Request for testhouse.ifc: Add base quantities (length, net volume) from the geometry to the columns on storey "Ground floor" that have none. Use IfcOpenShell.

First a look at what the model holds.

```python
import ifcopenshell
import ifcopenshell.util.element
import ifcopenshell.util.unit

model = ifcopenshell.open("testhouse.ifc")
print(model.schema)
for unit_type in ("LENGTHUNIT", "AREAUNIT", "VOLUMEUNIT"):
    print(unit_type, ifcopenshell.util.unit.calculate_unit_scale(model, unit_type))
storey = next(s for s in model.by_type("IfcBuildingStorey") if s.Name == "Ground floor")
columns = [e for e in ifcopenshell.util.element.get_decomposition(storey) if e.is_a("IfcColumn")]
for e in sorted(columns, key=lambda e: e.id()):
    print(e.id(), e.is_a(), e.Name, list(ifcopenshell.util.element.get_psets(e, qtos_only=True)), sep=" | ")
```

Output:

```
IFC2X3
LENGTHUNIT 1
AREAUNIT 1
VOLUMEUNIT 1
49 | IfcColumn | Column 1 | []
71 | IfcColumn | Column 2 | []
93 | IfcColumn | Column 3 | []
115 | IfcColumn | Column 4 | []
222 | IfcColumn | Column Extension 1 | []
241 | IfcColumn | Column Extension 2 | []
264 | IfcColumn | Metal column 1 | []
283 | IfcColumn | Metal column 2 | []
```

```python
import ifcopenshell
import ifcopenshell.api.pset
import ifcopenshell.geom
import ifcopenshell.util.element
import ifcopenshell.util.shape
import ifcopenshell.util.unit

model = ifcopenshell.open("testhouse.ifc")
unit_scale = ifcopenshell.util.unit.calculate_unit_scale(model)
volume_scale = ifcopenshell.util.unit.calculate_unit_scale(model, "VOLUMEUNIT")
settings = ifcopenshell.geom.settings()

storey = next(s for s in model.by_type("IfcBuildingStorey") if s.Name == "Ground floor")
columns = [e for e in ifcopenshell.util.element.get_decomposition(storey) if e.is_a("IfcColumn")]

for e in sorted(columns, key=lambda e: e.id()):
    if ifcopenshell.util.element.get_psets(e, qtos_only=True, should_inherit=False):
        continue
    # Geometry comes back in metres, in the element's own axes.
    shape = ifcopenshell.geom.create_shape(settings, e)
    values = {
        "Length": ifcopenshell.util.shape.get_z(shape.geometry) / unit_scale,
        "NetVolume": ifcopenshell.util.shape.get_volume(shape.geometry) / volume_scale,
    }
    qto = ifcopenshell.api.pset.add_qto(model, product=e, name="BaseQuantities")
    ifcopenshell.api.pset.edit_qto(model, qto=qto, properties=values)
    print(e.id(), {k: round(v, 3) for k, v in values.items()})

model.write("testhouse-out.ifc")
```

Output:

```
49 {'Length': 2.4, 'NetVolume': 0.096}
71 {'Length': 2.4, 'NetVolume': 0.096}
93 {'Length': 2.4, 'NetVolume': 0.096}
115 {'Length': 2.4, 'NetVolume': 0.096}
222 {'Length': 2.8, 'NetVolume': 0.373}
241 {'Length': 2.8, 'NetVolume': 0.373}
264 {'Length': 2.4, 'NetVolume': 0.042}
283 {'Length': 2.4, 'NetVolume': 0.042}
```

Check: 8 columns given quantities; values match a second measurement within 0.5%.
